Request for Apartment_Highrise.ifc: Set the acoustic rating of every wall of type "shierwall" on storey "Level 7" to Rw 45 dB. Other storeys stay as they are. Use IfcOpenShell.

First a look at what the model holds.

```python
import ifcopenshell
import ifcopenshell.util.element

model = ifcopenshell.open("Apartment_Highrise.ifc")
print(model.schema)
storey = next(s for s in model.by_type("IfcBuildingStorey") if s.Name == "Level 7")
walls = [e for e in ifcopenshell.util.element.get_decomposition(storey) if e.is_a("IfcWall")]
seen = {}
for e in walls:
    element_type = ifcopenshell.util.element.get_type(e)
    key = (element_type.Name if element_type != e and element_type else None, ifcopenshell.util.element.get_pset(e, "Pset_WallCommon", "AcousticRating"))
    seen[key] = seen.get(key, 0) + 1
for (name, value), count in sorted(seen.items(), key=str):
    print(count, "x", name, "|", value)
```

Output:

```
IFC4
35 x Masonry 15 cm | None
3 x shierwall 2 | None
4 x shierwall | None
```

```python
import ifcopenshell
import ifcopenshell.api.pset
import ifcopenshell.util.element

model = ifcopenshell.open("Apartment_Highrise.ifc")

storey = next(s for s in model.by_type("IfcBuildingStorey") if s.Name == "Level 7")
walls = [e for e in ifcopenshell.util.element.get_decomposition(storey) if e.is_a("IfcWall")]

count = 0
for e in walls:
    element_type = ifcopenshell.util.element.get_type(e)
    if element_type in (None, e) or element_type.Name != "shierwall":
        continue
    # add_pset returns the element's existing set when there is one.
    pset = ifcopenshell.api.pset.add_pset(model, product=e, name="Pset_WallCommon")
    ifcopenshell.api.pset.edit_pset(model, pset=pset, properties={"AcousticRating": "Rw 45 dB"})
    count += 1

print(count, "walls updated")

model.write("Apartment_Highrise_edited.ifc")
```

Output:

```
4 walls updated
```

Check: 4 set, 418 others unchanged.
